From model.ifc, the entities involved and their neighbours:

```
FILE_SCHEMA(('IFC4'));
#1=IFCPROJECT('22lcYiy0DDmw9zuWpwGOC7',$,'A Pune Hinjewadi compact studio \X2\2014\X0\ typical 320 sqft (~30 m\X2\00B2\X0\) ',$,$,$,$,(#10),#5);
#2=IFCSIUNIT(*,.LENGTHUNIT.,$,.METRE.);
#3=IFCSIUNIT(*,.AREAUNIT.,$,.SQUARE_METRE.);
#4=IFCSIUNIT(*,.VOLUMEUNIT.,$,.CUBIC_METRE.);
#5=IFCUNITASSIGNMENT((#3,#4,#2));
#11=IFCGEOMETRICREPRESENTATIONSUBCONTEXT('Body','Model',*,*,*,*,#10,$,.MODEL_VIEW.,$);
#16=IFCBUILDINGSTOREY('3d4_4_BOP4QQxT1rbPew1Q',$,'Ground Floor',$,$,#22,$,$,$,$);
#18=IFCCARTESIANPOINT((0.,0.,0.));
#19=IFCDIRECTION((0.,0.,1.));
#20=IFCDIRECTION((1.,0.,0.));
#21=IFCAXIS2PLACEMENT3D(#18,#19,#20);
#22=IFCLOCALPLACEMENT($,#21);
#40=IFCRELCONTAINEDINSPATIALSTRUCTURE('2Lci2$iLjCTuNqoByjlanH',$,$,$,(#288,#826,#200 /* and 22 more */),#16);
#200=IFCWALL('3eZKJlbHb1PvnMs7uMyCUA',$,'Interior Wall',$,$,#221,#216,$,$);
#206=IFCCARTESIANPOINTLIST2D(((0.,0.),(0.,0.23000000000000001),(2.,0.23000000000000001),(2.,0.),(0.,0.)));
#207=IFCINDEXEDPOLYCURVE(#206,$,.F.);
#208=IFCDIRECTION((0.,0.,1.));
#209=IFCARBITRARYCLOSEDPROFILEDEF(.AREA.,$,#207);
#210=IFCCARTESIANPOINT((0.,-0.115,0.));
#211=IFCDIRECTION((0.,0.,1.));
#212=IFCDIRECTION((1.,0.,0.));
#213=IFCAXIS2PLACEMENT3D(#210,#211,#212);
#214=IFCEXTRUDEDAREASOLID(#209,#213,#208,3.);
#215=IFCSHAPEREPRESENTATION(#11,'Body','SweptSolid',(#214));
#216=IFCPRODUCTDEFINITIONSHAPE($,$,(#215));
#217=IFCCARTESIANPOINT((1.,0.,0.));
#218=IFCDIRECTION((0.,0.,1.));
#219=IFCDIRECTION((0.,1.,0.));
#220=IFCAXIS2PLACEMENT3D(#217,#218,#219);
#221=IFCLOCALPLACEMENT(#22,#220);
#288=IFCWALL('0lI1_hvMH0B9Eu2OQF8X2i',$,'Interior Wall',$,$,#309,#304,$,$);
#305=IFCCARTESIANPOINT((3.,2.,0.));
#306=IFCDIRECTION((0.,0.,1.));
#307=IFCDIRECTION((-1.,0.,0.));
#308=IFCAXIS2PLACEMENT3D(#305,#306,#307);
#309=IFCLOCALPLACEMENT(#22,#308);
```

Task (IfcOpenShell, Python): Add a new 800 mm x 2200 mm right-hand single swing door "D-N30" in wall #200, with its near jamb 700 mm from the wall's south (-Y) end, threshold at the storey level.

```python
import numpy as np
import ifcopenshell
import ifcopenshell.api.feature
import ifcopenshell.api.geometry
import ifcopenshell.api.root
import ifcopenshell.api.spatial
import ifcopenshell.geom
import ifcopenshell.util.element
import ifcopenshell.util.placement
import ifcopenshell.util.representation
import ifcopenshell.util.shape
import ifcopenshell.util.unit

model = ifcopenshell.open("model.ifc")
unit_scale = ifcopenshell.util.unit.calculate_unit_scale(model)
settings = ifcopenshell.geom.settings()


def volume(element):
    """Net volume in cubic metres, openings subtracted."""
    shape = ifcopenshell.geom.create_shape(settings, element)
    return ifcopenshell.util.shape.get_volume(shape.geometry)


wall = model.by_guid("3eZKJlbHb1PvnMs7uMyCUA")
storey = ifcopenshell.util.element.get_container(wall, ifc_class="IfcBuildingStorey")
context = ifcopenshell.util.representation.get_context(model, "Model", "Body", "MODEL_VIEW")
before = volume(wall)

width, height, from_end, sill = 0.8, 2.2, 0.7, 0.0  # metres

# The wall runs along its own X axis, and the end named is its -X end.
wall_shape = ifcopenshell.geom.create_shape(settings, wall)
x, y, z = ifcopenshell.util.shape.get_vertices(wall_shape.geometry).T
start = x.min() + from_end
face, thickness = float(y.min()), float(y.max() - y.min())
wall_matrix = ifcopenshell.util.placement.get_local_placement(wall.ObjectPlacement)
level = ifcopenshell.util.placement.get_local_placement(storey.ObjectPlacement)[2, 3]


def in_wall(x, y):
    """Placement at x, y metres in the wall's axes, at sill height."""
    matrix = wall_matrix.copy()
    matrix[:, 3] = wall_matrix @ np.array([x / unit_scale, y / unit_scale, 0.0, 1.0])
    matrix[2, 3] = level + sill / unit_scale
    return matrix


# Opening: a box that overshoots both wall faces by 50 mm.
opening = ifcopenshell.api.root.create_entity(model, ifc_class="IfcOpeningElement", predefined_type="OPENING")
box = ifcopenshell.api.geometry.add_wall_representation(
    model, context=context, length=width, height=height, thickness=thickness + 0.1
)
ifcopenshell.api.geometry.assign_representation(model, product=opening, representation=box)
ifcopenshell.api.geometry.edit_object_placement(model, product=opening, matrix=in_wall(start, face - 0.05), is_si=False)
ifcopenshell.api.feature.add_feature(model, feature=opening, element=wall)

door = ifcopenshell.api.root.create_entity(model, ifc_class="IfcDoor", name="D-N30", predefined_type="DOOR")
door.OverallWidth, door.OverallHeight = width / unit_scale, height / unit_scale
door.OperationType = "SINGLE_SWING_RIGHT"
body = ifcopenshell.api.geometry.add_door_representation(
    model,
    context=context,
    overall_width=door.OverallWidth,
    overall_height=door.OverallHeight,
    operation_type="SINGLE_SWING_RIGHT",
    lining_properties={"LiningDepth": thickness / unit_scale, "ThresholdDepth": thickness / unit_scale},
)
ifcopenshell.api.geometry.assign_representation(model, product=door, representation=body)
ifcopenshell.api.spatial.assign_container(model, products=[door], relating_structure=storey)
ifcopenshell.api.feature.add_filling(model, opening=opening, element=door)

# The lining spans the wall, so the door starts at the wall face.
ifcopenshell.api.geometry.edit_object_placement(model, product=door, matrix=in_wall(start, face), is_si=False)

after = volume(wall)

print(f"wall volume {before:.3f} -> {after:.3f} m3")

model.write("model_updated.ifc")
```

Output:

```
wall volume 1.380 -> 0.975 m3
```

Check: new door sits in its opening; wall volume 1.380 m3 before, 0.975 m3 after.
